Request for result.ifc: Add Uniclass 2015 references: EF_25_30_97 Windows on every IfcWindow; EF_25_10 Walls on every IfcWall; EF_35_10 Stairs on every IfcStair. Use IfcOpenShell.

First a look at what the model holds.

```python
import ifcopenshell

model = ifcopenshell.open("result.ifc")
print(model.schema)
print("classifications:", [c.Name for c in model.by_type("IfcClassification")])
for ifc_class in ("IfcDoor", "IfcRoof", "IfcStair", "IfcWall", "IfcWindow"):
    print(ifc_class, len(model.by_type(ifc_class)))
```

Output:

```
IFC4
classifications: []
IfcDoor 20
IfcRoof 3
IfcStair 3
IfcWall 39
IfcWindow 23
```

```python
import ifcopenshell
import ifcopenshell.api.classification

model = ifcopenshell.open("result.ifc")

system = ifcopenshell.api.classification.add_classification(model, classification="Uniclass 2015")

codes = {
    "IfcWindow": ("EF_25_30_97", "Windows"),
    "IfcWall": ("EF_25_10", "Walls"),
    "IfcStair": ("EF_35_10", "Stairs"),
}
for ifc_class, (code, name) in codes.items():
    products = model.by_type(ifc_class)
    ifcopenshell.api.classification.add_reference(
        model, products=products, classification=system, identification=code, name=name
    )
    print(code, len(products))

model.write("result-out.ifc")
```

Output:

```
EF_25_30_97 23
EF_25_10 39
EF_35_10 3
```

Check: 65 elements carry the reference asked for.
